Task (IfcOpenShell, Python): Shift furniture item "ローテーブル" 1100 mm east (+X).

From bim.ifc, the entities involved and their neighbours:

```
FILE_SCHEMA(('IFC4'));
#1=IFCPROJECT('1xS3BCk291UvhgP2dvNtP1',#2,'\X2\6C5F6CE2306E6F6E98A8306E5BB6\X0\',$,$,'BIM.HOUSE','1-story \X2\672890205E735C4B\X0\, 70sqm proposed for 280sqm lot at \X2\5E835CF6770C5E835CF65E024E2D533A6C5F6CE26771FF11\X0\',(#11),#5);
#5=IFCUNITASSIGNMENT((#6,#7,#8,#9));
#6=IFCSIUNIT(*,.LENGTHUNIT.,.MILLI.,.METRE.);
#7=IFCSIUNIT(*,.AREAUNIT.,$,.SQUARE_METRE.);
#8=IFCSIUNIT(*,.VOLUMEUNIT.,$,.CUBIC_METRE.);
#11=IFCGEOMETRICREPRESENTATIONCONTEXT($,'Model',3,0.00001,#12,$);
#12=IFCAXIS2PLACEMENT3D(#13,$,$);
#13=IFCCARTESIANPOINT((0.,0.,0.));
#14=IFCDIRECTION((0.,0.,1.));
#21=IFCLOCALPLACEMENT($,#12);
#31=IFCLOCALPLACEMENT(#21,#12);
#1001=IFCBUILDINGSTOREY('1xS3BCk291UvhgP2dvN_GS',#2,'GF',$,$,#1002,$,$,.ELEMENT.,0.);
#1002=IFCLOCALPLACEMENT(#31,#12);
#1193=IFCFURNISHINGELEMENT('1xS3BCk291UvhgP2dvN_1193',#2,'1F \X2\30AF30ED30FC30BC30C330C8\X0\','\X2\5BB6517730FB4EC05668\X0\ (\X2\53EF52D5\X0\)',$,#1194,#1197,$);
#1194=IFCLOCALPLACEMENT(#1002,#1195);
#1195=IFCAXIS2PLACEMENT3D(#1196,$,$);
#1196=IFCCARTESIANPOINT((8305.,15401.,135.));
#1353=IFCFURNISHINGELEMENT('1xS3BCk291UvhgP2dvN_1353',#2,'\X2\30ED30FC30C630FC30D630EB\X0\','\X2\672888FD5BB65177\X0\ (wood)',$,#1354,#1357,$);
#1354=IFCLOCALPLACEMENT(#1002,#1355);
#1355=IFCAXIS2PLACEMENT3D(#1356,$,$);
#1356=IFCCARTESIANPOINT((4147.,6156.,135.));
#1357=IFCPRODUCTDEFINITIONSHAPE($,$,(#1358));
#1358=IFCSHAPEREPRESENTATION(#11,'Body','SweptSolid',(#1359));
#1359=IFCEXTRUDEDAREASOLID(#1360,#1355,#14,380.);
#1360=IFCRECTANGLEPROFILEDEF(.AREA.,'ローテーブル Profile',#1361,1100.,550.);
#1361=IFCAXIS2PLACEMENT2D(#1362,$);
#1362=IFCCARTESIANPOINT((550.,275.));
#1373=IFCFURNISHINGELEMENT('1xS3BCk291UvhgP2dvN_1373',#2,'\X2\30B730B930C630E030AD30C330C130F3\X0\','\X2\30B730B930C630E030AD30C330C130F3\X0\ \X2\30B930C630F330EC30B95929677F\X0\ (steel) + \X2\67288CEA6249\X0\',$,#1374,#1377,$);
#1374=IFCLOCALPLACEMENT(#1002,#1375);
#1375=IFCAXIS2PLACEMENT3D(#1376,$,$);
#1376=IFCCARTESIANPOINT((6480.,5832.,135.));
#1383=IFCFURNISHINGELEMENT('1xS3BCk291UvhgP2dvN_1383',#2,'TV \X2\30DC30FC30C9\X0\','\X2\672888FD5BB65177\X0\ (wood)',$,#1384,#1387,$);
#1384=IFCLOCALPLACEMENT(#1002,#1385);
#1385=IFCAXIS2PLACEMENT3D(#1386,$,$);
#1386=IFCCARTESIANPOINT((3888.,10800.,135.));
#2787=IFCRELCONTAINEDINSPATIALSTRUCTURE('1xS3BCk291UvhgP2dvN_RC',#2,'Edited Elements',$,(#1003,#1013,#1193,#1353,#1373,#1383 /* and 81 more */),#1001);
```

```python
import ifcopenshell
import ifcopenshell.api.geometry
import ifcopenshell.util.placement
import ifcopenshell.util.unit

model = ifcopenshell.open("bim.ifc")
unit_scale = ifcopenshell.util.unit.calculate_unit_scale(model)

item = model.by_guid("1xS3BCk291UvhgP2dvN_1353")
matrix = ifcopenshell.util.placement.get_local_placement(item.ObjectPlacement)
matrix[0, 3] += 1.1 / unit_scale
ifcopenshell.api.geometry.edit_object_placement(model, product=item, matrix=matrix, is_si=False)

print(ifcopenshell.util.placement.get_local_placement(item.ObjectPlacement).round(3) + 0.0)

model.write("bim_rev.ifc")
```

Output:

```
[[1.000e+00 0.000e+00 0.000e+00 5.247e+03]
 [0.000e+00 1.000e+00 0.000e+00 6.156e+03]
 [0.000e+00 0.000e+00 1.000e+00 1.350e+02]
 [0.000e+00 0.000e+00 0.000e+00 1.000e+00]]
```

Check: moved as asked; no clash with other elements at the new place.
